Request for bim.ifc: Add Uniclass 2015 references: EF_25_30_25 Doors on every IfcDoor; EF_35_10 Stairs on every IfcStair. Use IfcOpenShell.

First a look at what the model holds.

```python
import ifcopenshell

model = ifcopenshell.open("bim.ifc")
print(model.schema)
print("classifications:", [c.Name for c in model.by_type("IfcClassification")])
for ifc_class in ("IfcDoor", "IfcRoof", "IfcStair", "IfcWall", "IfcWindow"):
    print(ifc_class, len(model.by_type(ifc_class)))
```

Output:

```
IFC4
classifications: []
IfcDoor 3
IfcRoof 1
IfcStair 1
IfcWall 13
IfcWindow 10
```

```python
import ifcopenshell
import ifcopenshell.api.classification

model = ifcopenshell.open("bim.ifc")

system = ifcopenshell.api.classification.add_classification(model, classification="Uniclass 2015")

codes = {
    "IfcDoor": ("EF_25_30_25", "Doors"),
    "IfcStair": ("EF_35_10", "Stairs"),
}
for ifc_class, (code, name) in codes.items():
    products = model.by_type(ifc_class)
    ifcopenshell.api.classification.add_reference(
        model, products=products, classification=system, identification=code, name=name
    )
    print(code, len(products))

model.write("bim_v2.ifc")
```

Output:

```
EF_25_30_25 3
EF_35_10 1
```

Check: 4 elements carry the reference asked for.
